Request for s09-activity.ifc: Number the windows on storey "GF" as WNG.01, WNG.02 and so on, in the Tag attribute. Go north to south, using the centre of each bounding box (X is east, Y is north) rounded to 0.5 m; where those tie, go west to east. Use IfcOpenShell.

First a look at what the model holds.

```python
import ifcopenshell
import ifcopenshell.util.element
import ifcopenshell.util.placement

model = ifcopenshell.open("s09-activity.ifc")
print(model.schema)
storey = next(s for s in model.by_type("IfcBuildingStorey") if s.Name == "GF")
windows = [e for e in ifcopenshell.util.element.get_decomposition(storey) if e.is_a("IfcWindow")]
for e in sorted(windows, key=lambda e: e.id()):
    origin = ifcopenshell.util.placement.get_local_placement(e.ObjectPlacement)[:3, 3]
    print(e.id(), e.Tag, e.Name, origin.round(2) + 0.0, sep=" | ")
```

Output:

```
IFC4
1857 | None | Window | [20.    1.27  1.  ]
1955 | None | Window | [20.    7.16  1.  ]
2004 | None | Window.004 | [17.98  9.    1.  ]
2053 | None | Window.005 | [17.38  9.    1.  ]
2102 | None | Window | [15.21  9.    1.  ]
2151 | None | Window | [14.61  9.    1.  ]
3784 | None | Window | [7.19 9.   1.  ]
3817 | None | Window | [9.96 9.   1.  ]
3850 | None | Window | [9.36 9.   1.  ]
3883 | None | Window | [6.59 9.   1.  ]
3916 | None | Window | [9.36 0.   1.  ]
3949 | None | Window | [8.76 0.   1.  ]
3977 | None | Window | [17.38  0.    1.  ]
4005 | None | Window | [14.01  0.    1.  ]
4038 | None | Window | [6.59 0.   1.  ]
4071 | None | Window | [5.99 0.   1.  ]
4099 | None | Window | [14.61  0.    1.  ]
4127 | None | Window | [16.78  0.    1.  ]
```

```python
import ifcopenshell
import ifcopenshell.geom
import ifcopenshell.util.element
import ifcopenshell.util.shape

model = ifcopenshell.open("s09-activity.ifc")
settings = ifcopenshell.geom.settings()
settings.set("use-world-coords", True)


def centre(element):
    shape = ifcopenshell.geom.create_shape(settings, element)
    return ifcopenshell.util.shape.get_bbox_centroid(shape.geometry)


storey = next(s for s in model.by_type("IfcBuildingStorey") if s.Name == "GF")
windows = [e for e in ifcopenshell.util.element.get_decomposition(storey) if e.is_a("IfcWindow")]

# Insertion points can sit at a corner or the storey origin, so sort by the geometry (in metres).
centres = {e: centre(e) for e in windows}
windows.sort(key=lambda e: (-round(centres[e][1] / 0.5), centres[e][0]))

for i, e in enumerate(windows, start=1):
    number = f"WNG.{i:02d}"
    e.Tag = number
    print(e.id(), number)

model.write("s09-activity_edited.ifc")
```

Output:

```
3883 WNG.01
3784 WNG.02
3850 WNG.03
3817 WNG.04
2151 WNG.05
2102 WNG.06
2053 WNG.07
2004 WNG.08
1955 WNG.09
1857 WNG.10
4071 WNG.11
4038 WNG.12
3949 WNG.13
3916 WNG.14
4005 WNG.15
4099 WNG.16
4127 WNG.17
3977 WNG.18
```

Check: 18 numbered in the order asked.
